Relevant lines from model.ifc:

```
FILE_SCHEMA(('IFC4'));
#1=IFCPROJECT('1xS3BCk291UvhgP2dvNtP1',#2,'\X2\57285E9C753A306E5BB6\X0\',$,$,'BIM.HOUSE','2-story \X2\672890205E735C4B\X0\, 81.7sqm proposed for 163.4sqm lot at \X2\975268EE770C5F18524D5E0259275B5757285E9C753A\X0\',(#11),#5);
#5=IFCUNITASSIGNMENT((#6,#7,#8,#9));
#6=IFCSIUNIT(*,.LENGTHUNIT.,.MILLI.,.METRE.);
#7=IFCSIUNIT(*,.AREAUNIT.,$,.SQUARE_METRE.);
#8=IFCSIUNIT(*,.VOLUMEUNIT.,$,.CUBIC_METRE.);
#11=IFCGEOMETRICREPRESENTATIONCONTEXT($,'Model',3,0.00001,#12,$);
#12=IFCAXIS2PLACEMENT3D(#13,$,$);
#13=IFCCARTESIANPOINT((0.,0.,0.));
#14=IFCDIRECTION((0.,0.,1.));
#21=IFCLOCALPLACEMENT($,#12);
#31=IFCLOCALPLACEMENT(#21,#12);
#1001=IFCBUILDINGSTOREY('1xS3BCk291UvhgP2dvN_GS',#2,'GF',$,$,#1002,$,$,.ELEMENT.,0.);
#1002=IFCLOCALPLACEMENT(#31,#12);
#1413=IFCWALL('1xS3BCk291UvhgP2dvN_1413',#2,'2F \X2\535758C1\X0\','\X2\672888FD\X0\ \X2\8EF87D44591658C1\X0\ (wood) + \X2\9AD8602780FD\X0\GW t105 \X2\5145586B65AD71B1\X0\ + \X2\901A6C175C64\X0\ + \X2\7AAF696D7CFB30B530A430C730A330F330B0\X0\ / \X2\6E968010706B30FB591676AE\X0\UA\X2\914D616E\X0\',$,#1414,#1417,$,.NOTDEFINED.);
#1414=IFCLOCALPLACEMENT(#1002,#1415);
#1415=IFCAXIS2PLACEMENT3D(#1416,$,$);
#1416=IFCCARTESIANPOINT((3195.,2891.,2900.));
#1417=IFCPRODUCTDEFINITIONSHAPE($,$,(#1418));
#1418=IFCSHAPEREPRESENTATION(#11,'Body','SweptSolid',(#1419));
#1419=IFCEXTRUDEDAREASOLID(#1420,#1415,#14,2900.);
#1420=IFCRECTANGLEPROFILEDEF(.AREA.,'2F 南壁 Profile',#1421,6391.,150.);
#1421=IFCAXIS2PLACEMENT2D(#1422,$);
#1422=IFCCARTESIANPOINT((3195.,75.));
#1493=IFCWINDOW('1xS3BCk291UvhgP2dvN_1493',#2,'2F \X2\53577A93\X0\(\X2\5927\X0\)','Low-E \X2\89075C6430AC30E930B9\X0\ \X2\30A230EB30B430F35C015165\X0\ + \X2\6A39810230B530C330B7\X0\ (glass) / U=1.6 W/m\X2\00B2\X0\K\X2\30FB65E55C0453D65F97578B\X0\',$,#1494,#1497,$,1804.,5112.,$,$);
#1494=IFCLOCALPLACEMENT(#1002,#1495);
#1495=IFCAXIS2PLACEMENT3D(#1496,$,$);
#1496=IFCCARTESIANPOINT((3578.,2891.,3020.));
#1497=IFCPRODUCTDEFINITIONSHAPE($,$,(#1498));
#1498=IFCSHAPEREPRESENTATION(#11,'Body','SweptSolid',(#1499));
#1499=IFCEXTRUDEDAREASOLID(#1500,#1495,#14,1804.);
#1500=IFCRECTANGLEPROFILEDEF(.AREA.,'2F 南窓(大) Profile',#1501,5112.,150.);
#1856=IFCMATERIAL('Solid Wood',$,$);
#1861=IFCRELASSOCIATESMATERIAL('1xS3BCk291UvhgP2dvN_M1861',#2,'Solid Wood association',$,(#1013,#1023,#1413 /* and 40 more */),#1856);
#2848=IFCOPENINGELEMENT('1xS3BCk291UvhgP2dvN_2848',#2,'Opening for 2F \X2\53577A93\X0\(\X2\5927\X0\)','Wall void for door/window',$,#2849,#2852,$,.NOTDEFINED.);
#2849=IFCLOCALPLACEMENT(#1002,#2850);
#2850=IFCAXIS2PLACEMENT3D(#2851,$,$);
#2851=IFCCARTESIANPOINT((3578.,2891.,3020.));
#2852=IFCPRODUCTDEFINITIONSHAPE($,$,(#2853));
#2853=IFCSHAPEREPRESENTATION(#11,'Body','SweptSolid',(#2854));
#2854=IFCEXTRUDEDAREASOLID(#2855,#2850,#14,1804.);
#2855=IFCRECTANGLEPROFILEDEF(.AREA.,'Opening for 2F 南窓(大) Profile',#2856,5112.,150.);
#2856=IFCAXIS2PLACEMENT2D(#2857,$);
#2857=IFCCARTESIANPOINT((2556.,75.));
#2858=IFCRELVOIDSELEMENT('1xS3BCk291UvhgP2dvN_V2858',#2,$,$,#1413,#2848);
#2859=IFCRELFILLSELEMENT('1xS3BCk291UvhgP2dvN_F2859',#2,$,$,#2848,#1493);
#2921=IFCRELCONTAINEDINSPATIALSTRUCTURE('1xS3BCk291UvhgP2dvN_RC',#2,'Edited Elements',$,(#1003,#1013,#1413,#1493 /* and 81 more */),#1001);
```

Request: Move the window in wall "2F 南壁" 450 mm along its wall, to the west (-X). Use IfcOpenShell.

```python
import ifcopenshell
import ifcopenshell.api.geometry
import ifcopenshell.util.placement
import ifcopenshell.util.unit

model = ifcopenshell.open("model.ifc")
unit_scale = ifcopenshell.util.unit.calculate_unit_scale(model)

window = model.by_id(1493)
opening = window.FillsVoids[0].RelatingOpeningElement
wall = opening.VoidsElements[0].RelatingBuildingElement

wall_matrix = ifcopenshell.util.placement.get_local_placement(wall.ObjectPlacement)
shift = wall_matrix[:3, 0] * -0.45 / unit_scale
before = ifcopenshell.util.placement.get_local_placement(window.ObjectPlacement)[:3, 3].copy()

# The window is not placed relative to its opening, so move both.
for product in (opening, window):
    matrix = ifcopenshell.util.placement.get_local_placement(product.ObjectPlacement)
    matrix[:3, 3] += shift
    ifcopenshell.api.geometry.edit_object_placement(model, product=product, matrix=matrix, is_si=False)

after = ifcopenshell.util.placement.get_local_placement(window.ObjectPlacement)[:3, 3]
print("window moved by", (after - before).round(3) + 0.0)

model.write("model_edited.ifc")
```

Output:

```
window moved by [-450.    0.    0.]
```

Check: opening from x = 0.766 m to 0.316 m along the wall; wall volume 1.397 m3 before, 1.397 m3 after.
